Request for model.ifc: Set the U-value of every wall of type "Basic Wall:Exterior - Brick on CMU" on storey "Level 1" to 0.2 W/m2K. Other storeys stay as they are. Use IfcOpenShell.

First a look at what the model holds.

```python
import ifcopenshell
import ifcopenshell.util.element

model = ifcopenshell.open("model.ifc")
print(model.schema)
storey = next(s for s in model.by_type("IfcBuildingStorey") if s.Name == "Level 1")
walls = [e for e in ifcopenshell.util.element.get_decomposition(storey) if e.is_a("IfcWall")]
seen = {}
for e in walls:
    element_type = ifcopenshell.util.element.get_type(e)
    key = (element_type.Name if element_type != e and element_type else None, ifcopenshell.util.element.get_pset(e, "Pset_WallCommon", "ThermalTransmittance"))
    seen[key] = seen.get(key, 0) + 1
for (name, value), count in sorted(seen.items(), key=str):
    print(count, "x", name, "|", value)
```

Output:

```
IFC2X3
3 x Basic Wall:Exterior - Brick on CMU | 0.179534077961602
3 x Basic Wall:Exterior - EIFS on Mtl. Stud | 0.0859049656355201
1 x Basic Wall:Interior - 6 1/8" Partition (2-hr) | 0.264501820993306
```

```python
import ifcopenshell
import ifcopenshell.api.pset
import ifcopenshell.util.element

model = ifcopenshell.open("model.ifc")

storey = next(s for s in model.by_type("IfcBuildingStorey") if s.Name == "Level 1")
walls = [e for e in ifcopenshell.util.element.get_decomposition(storey) if e.is_a("IfcWall")]

count = 0
for e in walls:
    element_type = ifcopenshell.util.element.get_type(e)
    if element_type in (None, e) or element_type.Name != "Basic Wall:Exterior - Brick on CMU":
        continue
    # add_pset returns the element's existing set when there is one.
    pset = ifcopenshell.api.pset.add_pset(model, product=e, name="Pset_WallCommon")
    ifcopenshell.api.pset.edit_pset(model, pset=pset, properties={"ThermalTransmittance": 0.2})
    count += 1

print(count, "walls updated")

model.write("model_updated.ifc")
```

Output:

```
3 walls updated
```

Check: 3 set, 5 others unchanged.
